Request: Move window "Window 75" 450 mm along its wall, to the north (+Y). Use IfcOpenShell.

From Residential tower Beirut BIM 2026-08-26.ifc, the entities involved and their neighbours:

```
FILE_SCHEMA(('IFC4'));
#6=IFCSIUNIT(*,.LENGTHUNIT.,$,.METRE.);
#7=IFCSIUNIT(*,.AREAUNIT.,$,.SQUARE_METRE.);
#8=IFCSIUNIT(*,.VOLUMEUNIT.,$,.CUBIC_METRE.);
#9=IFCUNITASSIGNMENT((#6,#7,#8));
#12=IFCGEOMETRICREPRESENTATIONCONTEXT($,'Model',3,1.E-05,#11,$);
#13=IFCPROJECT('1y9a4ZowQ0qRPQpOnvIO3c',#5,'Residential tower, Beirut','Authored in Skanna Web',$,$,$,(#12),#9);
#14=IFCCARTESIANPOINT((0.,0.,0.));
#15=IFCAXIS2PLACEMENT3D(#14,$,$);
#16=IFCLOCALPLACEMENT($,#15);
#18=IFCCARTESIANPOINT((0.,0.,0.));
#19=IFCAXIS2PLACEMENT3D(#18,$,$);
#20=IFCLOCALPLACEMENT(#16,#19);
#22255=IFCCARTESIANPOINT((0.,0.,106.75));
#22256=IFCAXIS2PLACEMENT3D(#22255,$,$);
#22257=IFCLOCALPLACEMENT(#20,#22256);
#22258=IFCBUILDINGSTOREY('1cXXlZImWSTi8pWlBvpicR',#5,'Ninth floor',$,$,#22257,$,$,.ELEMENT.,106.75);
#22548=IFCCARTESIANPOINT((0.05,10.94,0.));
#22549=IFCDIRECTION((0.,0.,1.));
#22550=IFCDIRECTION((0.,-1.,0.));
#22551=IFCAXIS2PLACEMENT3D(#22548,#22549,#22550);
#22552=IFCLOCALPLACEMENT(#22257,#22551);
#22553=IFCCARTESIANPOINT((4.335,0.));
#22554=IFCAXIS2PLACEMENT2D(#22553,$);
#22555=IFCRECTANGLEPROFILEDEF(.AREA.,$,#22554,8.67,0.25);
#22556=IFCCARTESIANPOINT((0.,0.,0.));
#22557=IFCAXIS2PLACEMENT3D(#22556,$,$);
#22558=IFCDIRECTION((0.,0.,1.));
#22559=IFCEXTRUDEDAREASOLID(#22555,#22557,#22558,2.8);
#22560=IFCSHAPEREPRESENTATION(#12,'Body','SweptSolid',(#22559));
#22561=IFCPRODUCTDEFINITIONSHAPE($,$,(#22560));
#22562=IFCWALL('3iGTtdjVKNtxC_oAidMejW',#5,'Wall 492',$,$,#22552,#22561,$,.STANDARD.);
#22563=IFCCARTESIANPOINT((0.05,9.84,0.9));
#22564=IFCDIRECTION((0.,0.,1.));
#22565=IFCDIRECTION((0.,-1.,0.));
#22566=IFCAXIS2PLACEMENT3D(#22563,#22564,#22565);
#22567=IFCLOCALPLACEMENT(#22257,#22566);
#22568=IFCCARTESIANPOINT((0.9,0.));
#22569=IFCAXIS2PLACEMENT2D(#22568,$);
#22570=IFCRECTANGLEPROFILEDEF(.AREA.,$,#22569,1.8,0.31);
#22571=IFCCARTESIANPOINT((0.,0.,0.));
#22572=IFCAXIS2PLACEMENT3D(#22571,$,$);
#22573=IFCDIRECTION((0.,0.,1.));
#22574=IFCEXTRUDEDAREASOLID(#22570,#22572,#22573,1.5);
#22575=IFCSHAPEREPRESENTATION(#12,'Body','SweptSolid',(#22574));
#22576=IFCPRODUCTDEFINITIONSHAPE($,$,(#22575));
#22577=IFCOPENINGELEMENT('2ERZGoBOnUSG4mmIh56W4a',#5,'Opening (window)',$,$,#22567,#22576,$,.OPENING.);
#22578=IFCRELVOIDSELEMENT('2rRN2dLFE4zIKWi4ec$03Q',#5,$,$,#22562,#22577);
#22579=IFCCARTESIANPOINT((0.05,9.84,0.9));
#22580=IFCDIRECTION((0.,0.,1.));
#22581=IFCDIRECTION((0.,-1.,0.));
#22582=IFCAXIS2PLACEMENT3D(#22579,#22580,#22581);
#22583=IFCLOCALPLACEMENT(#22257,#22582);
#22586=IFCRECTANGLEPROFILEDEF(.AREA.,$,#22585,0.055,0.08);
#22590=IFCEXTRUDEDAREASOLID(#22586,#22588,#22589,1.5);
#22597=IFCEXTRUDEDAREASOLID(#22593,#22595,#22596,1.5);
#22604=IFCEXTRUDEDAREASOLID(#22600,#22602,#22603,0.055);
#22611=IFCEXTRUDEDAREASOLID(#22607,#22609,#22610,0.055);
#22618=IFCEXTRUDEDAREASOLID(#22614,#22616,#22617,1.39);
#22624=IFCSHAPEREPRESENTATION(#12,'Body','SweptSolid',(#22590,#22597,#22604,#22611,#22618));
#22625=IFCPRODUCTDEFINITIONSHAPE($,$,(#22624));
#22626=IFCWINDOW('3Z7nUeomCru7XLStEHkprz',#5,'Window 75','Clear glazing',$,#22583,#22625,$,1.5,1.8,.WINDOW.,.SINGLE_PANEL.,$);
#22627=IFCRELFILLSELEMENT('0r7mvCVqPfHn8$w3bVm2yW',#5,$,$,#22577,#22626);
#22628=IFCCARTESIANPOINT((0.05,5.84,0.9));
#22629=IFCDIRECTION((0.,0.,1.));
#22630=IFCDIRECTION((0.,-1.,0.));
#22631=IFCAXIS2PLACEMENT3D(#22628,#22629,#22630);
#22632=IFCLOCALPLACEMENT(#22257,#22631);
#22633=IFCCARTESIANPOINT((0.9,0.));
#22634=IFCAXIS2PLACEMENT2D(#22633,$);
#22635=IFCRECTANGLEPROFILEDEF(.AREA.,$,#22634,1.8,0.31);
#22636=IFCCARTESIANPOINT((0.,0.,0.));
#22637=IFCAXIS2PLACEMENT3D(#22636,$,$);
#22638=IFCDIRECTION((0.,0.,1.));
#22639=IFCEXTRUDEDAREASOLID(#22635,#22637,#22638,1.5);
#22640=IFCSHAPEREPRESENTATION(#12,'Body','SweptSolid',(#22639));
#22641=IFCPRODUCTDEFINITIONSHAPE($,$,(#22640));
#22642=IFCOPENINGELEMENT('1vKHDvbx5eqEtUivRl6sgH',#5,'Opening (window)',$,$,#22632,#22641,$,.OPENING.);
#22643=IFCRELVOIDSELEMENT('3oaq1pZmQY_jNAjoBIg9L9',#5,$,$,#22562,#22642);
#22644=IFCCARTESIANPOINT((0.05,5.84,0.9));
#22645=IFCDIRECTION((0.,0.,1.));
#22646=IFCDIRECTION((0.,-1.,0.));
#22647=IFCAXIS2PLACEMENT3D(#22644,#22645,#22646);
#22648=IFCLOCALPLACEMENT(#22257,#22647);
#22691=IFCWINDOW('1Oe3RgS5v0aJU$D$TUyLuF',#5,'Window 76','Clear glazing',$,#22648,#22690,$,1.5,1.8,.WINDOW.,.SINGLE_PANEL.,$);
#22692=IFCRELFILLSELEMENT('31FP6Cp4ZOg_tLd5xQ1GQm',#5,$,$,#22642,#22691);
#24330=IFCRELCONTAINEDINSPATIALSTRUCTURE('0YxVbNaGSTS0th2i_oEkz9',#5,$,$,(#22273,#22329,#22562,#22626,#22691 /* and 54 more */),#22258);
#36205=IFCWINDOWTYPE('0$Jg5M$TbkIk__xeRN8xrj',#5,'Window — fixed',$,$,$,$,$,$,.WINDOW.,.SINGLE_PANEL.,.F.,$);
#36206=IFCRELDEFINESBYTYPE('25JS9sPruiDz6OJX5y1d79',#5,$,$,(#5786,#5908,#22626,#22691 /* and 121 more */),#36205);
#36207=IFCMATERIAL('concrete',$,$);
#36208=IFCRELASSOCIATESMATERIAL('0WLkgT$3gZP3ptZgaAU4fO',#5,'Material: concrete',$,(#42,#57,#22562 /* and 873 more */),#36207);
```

```python
import ifcopenshell
import ifcopenshell.api.geometry
import ifcopenshell.util.placement

model = ifcopenshell.open("Residential tower Beirut BIM 2026-08-26.ifc")

window = model.by_id(22626)
opening = window.FillsVoids[0].RelatingOpeningElement
wall = opening.VoidsElements[0].RelatingBuildingElement

wall_matrix = ifcopenshell.util.placement.get_local_placement(wall.ObjectPlacement)
shift = wall_matrix[:3, 0] * -0.45
before = ifcopenshell.util.placement.get_local_placement(window.ObjectPlacement)[:3, 3].copy()

# The window is not placed relative to its opening, so move both.
for product in (opening, window):
    matrix = ifcopenshell.util.placement.get_local_placement(product.ObjectPlacement)
    matrix[:3, 3] += shift
    ifcopenshell.api.geometry.edit_object_placement(model, product=product, matrix=matrix, is_si=False)

after = ifcopenshell.util.placement.get_local_placement(window.ObjectPlacement)[:3, 3]
print("window moved by", (after - before).round(3) + 0.0)

model.write("Residential tower Beirut BIM 2026-08-26-out.ifc")
```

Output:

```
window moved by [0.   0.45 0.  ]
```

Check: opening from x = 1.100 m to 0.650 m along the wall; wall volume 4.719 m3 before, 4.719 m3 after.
